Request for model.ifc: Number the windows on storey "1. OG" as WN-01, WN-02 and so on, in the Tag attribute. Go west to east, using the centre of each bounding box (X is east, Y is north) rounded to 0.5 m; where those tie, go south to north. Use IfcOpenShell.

First a look at what the model holds.

```python
import ifcopenshell
import ifcopenshell.util.element
import ifcopenshell.util.placement

model = ifcopenshell.open("model.ifc")
print(model.schema)
storey = next(s for s in model.by_type("IfcBuildingStorey") if s.Name == "1. OG")
windows = [e for e in ifcopenshell.util.element.get_decomposition(storey) if e.is_a("IfcWindow")]
for e in sorted(windows, key=lambda e: e.id()):
    origin = ifcopenshell.util.placement.get_local_placement(e.ObjectPlacement)[:3, 3]
    print(e.id(), e.Tag, e.Name, origin.round(2) + 0.0, sep=" | ")
```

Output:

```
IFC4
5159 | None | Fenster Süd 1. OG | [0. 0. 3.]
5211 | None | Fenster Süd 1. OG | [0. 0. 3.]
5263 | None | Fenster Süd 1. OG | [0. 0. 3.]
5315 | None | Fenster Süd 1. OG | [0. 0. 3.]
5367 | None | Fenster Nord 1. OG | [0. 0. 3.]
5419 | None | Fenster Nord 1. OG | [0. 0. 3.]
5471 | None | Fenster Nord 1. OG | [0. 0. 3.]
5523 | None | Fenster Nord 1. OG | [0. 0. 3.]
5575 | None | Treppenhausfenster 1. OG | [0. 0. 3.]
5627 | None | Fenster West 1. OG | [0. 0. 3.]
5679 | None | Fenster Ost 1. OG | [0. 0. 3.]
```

```python
import ifcopenshell
import ifcopenshell.geom
import ifcopenshell.util.element
import ifcopenshell.util.shape

model = ifcopenshell.open("model.ifc")
settings = ifcopenshell.geom.settings()
settings.set("use-world-coords", True)


def centre(element):
    shape = ifcopenshell.geom.create_shape(settings, element)
    return ifcopenshell.util.shape.get_bbox_centroid(shape.geometry)


storey = next(s for s in model.by_type("IfcBuildingStorey") if s.Name == "1. OG")
windows = [e for e in ifcopenshell.util.element.get_decomposition(storey) if e.is_a("IfcWindow")]

# Insertion points can sit at a corner or the storey origin, so sort by the geometry (in metres).
centres = {e: centre(e) for e in windows}
windows.sort(key=lambda e: (round(centres[e][0] / 0.5), centres[e][1]))

for i, e in enumerate(windows, start=1):
    number = f"WN-{i:02d}"
    e.Tag = number
    print(e.id(), number)

model.write("model_rev.ifc")
```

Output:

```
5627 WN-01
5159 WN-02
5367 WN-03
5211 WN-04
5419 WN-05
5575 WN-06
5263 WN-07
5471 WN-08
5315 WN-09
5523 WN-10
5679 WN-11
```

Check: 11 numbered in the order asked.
